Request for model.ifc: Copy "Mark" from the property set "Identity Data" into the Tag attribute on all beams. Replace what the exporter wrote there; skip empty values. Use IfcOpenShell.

First a look at what the model holds.

```python
import ifcopenshell
import ifcopenshell.util.element

model = ifcopenshell.open("model.ifc")
print(model.schema)
beams = model.by_type("IfcBeam")
print(len(beams), "beams")
for e in beams[:8]:
    source = ifcopenshell.util.element.get_pset(e, "Identity Data", "Mark")
    target = e.Tag
    print(e.id(), repr(source), repr(target), sep=" | ")
```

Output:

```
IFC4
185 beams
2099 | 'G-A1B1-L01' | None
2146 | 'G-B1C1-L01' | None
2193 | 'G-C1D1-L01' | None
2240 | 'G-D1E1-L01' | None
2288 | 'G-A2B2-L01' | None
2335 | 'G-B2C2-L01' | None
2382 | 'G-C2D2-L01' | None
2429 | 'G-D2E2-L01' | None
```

```python
import ifcopenshell
import ifcopenshell.util.element

model = ifcopenshell.open("model.ifc")

count = 0
for e in model.by_type("IfcBeam"):
    value = ifcopenshell.util.element.get_pset(e, "Identity Data", "Mark")
    current = e.Tag
    if not value or not value.strip() or current == value:
        continue
    e.Tag = value
    count += 1

print(count, "beams updated")

model.write("model_v2.ifc")
```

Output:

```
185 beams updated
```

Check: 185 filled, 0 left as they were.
